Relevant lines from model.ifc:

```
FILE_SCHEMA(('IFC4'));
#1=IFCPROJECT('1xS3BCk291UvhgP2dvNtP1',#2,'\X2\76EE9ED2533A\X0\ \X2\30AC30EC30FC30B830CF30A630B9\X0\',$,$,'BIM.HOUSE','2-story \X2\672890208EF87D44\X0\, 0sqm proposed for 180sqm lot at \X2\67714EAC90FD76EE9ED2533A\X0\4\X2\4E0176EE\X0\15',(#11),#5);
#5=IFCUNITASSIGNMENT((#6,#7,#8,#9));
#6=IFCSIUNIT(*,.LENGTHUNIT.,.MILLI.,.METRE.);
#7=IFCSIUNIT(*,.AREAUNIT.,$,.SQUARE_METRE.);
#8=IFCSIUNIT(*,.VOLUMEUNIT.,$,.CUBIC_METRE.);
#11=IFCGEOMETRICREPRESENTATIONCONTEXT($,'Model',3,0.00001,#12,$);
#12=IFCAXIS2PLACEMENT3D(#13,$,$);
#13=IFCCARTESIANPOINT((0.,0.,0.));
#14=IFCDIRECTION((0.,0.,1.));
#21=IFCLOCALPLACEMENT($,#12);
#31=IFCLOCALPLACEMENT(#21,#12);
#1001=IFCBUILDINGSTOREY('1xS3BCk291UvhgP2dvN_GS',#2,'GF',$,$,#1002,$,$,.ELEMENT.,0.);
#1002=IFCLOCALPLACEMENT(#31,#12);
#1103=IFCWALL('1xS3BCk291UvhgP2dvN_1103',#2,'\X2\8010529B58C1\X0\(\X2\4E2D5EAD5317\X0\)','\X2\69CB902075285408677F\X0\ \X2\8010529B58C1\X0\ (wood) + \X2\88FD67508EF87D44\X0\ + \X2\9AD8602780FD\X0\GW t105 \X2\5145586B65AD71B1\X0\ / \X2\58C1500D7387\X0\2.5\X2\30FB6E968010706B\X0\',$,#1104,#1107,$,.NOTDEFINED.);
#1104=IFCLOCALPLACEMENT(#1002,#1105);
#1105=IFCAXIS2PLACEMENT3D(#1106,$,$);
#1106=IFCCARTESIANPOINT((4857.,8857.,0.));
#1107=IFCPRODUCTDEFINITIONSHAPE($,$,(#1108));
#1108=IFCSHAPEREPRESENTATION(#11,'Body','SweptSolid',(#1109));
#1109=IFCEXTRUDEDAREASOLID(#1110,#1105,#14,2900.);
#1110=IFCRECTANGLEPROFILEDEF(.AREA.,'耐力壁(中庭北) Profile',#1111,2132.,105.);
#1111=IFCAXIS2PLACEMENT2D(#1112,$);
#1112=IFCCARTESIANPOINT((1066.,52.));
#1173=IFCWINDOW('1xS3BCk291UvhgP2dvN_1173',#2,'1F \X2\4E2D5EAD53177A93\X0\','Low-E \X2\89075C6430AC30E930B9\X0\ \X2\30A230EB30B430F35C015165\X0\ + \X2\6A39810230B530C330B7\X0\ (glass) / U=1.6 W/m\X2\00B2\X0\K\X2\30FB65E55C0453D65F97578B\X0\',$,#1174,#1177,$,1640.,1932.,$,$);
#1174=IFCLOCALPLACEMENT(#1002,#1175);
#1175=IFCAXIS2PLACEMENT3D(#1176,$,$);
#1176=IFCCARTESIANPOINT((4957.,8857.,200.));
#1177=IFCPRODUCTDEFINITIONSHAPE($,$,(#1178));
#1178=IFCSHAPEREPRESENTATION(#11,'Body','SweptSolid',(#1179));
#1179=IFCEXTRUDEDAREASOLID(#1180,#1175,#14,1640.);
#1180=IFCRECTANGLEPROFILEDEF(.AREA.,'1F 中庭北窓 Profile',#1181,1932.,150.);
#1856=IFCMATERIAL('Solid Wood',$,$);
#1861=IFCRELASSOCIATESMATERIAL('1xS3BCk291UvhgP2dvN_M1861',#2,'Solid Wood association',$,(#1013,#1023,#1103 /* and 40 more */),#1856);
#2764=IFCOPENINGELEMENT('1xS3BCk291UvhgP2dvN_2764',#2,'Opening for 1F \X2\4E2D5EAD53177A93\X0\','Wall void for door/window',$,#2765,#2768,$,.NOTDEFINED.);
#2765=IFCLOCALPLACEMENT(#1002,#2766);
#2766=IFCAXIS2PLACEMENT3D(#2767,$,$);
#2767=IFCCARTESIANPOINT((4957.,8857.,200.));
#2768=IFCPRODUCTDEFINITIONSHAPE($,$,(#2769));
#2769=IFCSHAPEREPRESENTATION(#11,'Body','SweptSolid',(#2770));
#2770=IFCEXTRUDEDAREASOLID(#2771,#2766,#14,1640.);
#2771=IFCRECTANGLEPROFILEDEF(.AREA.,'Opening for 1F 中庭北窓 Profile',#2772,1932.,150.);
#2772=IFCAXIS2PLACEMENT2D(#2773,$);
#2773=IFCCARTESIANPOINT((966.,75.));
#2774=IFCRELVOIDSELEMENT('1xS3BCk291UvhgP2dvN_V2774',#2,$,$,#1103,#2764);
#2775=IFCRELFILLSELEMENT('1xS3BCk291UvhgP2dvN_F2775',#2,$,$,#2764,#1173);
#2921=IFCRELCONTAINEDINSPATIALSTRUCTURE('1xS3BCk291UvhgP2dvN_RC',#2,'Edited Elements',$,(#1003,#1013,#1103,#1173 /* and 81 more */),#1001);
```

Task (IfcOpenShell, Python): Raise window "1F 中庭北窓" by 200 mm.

```python
import numpy as np
import ifcopenshell
import ifcopenshell.api.geometry
import ifcopenshell.util.placement
import ifcopenshell.util.unit

model = ifcopenshell.open("model.ifc")
unit_scale = ifcopenshell.util.unit.calculate_unit_scale(model)

window = model.by_guid("1xS3BCk291UvhgP2dvN_1173")
opening = window.FillsVoids[0].RelatingOpeningElement
dz = 0.2 / unit_scale

shift = np.array([0.0, 0.0, dz])
# The window is not placed relative to its opening, so move both.
for product in (opening, window):
    matrix = ifcopenshell.util.placement.get_local_placement(product.ObjectPlacement)
    matrix[:3, 3] += shift
    ifcopenshell.api.geometry.edit_object_placement(model, product=product, matrix=matrix, is_si=False)

print(f"moved by {dz * unit_scale:+.3f} m")

model.write("model_rev.ifc")
```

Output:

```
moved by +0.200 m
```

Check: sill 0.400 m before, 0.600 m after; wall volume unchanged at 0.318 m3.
